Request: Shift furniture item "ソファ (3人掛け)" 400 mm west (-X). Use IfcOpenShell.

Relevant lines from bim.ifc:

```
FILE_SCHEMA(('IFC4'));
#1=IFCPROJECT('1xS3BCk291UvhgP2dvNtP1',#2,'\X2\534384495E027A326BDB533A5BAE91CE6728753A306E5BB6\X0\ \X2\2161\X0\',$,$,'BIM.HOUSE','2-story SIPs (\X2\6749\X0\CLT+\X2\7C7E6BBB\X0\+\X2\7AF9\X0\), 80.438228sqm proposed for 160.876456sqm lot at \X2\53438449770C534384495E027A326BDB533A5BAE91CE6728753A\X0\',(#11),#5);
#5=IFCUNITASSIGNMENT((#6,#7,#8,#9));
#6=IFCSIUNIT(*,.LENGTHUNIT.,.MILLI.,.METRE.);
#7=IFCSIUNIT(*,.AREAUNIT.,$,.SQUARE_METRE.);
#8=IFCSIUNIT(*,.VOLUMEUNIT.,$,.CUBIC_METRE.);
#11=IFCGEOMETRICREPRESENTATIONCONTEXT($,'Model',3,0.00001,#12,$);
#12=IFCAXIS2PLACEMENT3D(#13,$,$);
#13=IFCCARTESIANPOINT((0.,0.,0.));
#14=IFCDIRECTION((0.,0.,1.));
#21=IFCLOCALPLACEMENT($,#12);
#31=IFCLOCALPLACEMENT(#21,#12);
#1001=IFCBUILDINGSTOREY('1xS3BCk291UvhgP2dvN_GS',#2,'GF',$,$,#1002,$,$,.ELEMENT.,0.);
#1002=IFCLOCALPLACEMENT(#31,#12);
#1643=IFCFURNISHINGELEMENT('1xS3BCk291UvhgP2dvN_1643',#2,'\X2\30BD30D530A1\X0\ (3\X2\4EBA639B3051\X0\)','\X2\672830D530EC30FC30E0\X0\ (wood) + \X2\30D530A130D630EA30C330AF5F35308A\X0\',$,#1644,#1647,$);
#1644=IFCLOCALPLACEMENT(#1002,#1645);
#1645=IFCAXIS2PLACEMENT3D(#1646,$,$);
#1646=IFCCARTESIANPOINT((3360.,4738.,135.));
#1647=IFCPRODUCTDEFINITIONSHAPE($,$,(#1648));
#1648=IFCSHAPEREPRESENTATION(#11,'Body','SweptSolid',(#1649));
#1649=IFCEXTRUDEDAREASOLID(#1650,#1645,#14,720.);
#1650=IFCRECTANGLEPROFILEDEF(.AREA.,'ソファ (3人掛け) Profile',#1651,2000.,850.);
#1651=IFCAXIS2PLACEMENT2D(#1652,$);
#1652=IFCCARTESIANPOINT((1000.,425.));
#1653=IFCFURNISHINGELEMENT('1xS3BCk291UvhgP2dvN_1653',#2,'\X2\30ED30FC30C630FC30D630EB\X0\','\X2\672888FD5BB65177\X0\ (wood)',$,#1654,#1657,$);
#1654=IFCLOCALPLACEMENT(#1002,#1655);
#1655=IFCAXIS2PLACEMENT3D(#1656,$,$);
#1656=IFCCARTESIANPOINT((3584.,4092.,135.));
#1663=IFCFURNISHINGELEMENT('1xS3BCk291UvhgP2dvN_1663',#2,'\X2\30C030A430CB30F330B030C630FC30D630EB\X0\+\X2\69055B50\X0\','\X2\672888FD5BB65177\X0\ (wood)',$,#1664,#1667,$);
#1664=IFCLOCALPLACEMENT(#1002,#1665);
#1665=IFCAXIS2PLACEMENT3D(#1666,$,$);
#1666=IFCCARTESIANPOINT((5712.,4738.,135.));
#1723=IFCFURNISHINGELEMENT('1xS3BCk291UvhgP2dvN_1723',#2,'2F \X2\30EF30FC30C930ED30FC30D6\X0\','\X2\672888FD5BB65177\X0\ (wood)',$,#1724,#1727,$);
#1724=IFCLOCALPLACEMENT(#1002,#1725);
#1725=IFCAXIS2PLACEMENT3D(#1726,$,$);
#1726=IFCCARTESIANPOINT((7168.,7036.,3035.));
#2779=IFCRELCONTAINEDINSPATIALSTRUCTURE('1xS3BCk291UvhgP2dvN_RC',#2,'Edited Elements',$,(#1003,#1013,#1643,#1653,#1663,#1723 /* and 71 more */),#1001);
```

```python
import ifcopenshell
import ifcopenshell.api.geometry
import ifcopenshell.util.placement
import ifcopenshell.util.unit

model = ifcopenshell.open("bim.ifc")
unit_scale = ifcopenshell.util.unit.calculate_unit_scale(model)

item = model.by_guid("1xS3BCk291UvhgP2dvN_1643")
matrix = ifcopenshell.util.placement.get_local_placement(item.ObjectPlacement)
matrix[0, 3] -= 0.4 / unit_scale
ifcopenshell.api.geometry.edit_object_placement(model, product=item, matrix=matrix, is_si=False)

print(ifcopenshell.util.placement.get_local_placement(item.ObjectPlacement).round(3) + 0.0)

model.write("bim_v2.ifc")
```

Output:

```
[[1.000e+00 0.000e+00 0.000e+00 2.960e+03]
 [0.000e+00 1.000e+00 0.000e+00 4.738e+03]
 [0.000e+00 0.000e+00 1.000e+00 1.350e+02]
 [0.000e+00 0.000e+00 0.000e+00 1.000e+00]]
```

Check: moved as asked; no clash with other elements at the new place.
